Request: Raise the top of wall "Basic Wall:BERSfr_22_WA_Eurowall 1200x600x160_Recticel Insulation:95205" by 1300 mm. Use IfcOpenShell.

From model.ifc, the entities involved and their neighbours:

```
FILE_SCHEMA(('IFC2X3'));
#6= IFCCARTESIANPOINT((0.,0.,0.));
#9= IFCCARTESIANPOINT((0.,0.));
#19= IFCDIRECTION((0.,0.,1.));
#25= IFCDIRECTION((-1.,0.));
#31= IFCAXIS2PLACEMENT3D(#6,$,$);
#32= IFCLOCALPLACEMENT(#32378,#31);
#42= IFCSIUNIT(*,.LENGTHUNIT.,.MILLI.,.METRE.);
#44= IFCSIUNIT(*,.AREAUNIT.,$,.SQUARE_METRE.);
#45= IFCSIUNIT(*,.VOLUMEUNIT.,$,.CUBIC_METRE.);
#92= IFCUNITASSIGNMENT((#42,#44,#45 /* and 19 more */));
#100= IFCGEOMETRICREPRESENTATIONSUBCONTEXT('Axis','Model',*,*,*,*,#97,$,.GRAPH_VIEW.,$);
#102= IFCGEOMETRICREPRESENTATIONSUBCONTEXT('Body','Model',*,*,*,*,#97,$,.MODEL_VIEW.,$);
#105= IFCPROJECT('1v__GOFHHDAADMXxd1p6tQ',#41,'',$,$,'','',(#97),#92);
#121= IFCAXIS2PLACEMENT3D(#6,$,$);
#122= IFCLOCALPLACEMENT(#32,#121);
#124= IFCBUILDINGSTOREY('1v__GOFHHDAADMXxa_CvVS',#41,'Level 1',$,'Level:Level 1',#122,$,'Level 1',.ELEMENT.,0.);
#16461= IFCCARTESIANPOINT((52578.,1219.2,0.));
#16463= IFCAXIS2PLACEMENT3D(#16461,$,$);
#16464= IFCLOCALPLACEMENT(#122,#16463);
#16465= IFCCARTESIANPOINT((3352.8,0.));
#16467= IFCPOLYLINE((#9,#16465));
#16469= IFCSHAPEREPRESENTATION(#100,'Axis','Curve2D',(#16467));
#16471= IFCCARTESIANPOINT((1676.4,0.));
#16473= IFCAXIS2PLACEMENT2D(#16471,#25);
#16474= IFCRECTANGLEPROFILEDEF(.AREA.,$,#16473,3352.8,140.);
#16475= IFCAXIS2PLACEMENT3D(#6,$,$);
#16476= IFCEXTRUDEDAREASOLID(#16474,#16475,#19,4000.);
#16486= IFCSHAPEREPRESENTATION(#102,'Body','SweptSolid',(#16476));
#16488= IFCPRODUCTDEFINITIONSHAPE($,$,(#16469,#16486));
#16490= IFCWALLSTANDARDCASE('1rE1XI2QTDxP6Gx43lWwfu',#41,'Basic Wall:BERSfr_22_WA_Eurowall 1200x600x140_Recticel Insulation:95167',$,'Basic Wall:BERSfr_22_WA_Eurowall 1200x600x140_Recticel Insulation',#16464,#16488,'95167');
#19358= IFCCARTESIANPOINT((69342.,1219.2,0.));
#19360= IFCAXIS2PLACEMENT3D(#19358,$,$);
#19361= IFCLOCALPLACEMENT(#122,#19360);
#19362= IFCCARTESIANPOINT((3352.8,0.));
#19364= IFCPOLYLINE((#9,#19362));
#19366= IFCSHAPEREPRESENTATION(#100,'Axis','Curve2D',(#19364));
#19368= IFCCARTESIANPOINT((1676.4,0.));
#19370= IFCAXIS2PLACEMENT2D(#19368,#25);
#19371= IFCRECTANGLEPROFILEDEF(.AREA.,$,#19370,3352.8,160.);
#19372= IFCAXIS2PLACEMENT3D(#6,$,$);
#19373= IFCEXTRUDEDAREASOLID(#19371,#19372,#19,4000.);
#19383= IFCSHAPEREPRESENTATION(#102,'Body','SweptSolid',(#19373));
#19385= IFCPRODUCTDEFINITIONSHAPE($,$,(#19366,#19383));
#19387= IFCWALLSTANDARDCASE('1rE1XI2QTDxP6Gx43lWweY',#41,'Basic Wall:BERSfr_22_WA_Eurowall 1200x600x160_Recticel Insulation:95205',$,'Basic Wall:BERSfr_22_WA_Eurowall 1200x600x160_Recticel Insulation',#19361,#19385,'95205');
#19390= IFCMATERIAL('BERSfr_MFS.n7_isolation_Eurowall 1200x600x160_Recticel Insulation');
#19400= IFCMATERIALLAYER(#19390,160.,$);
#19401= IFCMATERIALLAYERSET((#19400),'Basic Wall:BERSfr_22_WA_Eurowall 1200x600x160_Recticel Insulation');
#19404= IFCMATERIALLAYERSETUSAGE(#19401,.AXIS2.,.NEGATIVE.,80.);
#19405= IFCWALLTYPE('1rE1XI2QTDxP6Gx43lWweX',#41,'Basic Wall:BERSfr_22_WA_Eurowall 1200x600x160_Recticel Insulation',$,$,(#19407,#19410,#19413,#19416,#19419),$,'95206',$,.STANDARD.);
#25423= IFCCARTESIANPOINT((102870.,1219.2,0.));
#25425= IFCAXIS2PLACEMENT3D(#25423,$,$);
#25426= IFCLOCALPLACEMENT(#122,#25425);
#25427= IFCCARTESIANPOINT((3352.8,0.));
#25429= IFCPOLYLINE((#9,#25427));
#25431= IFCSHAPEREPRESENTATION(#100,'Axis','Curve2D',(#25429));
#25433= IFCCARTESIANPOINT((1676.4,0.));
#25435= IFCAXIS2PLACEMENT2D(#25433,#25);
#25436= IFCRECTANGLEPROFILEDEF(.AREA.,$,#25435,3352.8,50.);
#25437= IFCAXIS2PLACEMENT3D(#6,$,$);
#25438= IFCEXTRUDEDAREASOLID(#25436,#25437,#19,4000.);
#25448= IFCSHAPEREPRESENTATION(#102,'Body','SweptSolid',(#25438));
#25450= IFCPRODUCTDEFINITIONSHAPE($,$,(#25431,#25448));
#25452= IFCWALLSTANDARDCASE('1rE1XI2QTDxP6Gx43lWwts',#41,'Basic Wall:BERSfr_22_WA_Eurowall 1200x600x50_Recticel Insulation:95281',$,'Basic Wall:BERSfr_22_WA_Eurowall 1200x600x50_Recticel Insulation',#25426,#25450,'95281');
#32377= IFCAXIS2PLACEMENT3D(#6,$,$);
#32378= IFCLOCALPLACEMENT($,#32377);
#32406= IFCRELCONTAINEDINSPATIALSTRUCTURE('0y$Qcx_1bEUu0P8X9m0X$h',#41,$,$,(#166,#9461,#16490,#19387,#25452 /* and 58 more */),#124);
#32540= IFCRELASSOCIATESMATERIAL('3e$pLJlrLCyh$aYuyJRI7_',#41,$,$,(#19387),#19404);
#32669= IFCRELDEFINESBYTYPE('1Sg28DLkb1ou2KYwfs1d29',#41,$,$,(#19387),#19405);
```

```python
import ifcopenshell
import ifcopenshell.geom
import ifcopenshell.util.representation
import ifcopenshell.util.shape
import ifcopenshell.util.unit

model = ifcopenshell.open("model.ifc")
unit_scale = ifcopenshell.util.unit.calculate_unit_scale(model)
settings = ifcopenshell.geom.settings()


def volume(element):
    """Net volume in cubic metres, openings subtracted."""
    shape = ifcopenshell.geom.create_shape(settings, element)
    return ifcopenshell.util.shape.get_volume(shape.geometry)


wall = model.by_guid("1rE1XI2QTDxP6Gx43lWweY")
before = volume(wall)

body = ifcopenshell.util.representation.get_representation(wall, "Model", "Body")
solid = body.Items[0]
old_height = solid.Depth
solid.Depth += 1.3 / unit_scale
after = volume(wall)

print(f"height {old_height:g} -> {solid.Depth:g}, volume {before:.3f} -> {after:.3f} m3")

model.write("model_v2.ifc")
```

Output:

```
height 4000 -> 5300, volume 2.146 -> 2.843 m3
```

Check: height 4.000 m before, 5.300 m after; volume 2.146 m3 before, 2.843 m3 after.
